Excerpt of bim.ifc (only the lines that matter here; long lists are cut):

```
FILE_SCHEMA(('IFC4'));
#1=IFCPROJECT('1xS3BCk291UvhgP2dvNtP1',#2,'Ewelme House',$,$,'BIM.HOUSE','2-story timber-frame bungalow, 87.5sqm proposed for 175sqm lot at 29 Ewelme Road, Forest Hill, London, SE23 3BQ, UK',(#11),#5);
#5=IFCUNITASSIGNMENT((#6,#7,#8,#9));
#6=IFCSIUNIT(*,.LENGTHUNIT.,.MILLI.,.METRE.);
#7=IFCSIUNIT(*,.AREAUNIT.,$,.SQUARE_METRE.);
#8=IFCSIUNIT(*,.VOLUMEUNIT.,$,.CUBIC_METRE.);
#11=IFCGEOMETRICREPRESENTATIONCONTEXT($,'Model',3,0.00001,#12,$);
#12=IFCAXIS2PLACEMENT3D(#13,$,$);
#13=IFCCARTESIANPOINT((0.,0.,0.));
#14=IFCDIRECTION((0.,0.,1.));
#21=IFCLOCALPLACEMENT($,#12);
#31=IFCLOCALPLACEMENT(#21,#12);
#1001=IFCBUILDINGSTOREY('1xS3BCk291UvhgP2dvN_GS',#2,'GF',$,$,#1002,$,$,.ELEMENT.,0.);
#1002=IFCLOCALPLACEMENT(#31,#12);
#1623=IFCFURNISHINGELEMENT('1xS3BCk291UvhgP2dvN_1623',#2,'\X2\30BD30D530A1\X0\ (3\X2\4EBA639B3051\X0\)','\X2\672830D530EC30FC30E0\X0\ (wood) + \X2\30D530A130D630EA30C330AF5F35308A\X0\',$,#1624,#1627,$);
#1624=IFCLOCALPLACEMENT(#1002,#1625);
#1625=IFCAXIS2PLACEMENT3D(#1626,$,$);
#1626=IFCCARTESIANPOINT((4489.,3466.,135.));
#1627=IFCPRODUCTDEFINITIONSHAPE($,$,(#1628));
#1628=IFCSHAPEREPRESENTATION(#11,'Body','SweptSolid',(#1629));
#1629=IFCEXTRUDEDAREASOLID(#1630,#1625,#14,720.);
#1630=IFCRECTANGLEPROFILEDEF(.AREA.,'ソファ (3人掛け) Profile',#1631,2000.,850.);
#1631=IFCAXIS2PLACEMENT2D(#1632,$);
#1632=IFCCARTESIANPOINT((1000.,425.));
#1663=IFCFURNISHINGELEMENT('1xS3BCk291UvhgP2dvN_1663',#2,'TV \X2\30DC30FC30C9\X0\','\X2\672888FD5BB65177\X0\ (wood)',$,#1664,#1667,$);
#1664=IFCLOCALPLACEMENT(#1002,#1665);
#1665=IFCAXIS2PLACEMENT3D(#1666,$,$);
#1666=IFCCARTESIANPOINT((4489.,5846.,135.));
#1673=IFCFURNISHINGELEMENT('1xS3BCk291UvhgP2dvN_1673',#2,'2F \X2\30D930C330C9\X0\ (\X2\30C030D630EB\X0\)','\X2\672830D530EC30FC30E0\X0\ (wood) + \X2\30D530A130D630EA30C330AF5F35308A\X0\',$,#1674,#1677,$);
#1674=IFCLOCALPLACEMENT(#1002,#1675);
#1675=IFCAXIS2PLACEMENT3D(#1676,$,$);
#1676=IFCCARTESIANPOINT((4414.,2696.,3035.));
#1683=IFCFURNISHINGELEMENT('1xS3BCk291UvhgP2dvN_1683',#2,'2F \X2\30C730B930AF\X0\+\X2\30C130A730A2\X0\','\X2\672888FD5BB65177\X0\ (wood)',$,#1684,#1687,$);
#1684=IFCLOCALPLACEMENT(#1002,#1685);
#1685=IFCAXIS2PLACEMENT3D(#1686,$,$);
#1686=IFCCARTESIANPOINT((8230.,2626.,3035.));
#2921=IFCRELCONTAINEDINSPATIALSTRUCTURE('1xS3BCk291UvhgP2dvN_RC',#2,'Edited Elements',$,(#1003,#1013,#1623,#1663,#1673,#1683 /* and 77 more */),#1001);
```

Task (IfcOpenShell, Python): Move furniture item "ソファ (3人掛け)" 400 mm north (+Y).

```python
import ifcopenshell
import ifcopenshell.api.geometry
import ifcopenshell.util.placement
import ifcopenshell.util.unit

model = ifcopenshell.open("bim.ifc")
unit_scale = ifcopenshell.util.unit.calculate_unit_scale(model)

item = model.by_guid("1xS3BCk291UvhgP2dvN_1623")
matrix = ifcopenshell.util.placement.get_local_placement(item.ObjectPlacement)
matrix[1, 3] += 0.4 / unit_scale
ifcopenshell.api.geometry.edit_object_placement(model, product=item, matrix=matrix, is_si=False)

print(ifcopenshell.util.placement.get_local_placement(item.ObjectPlacement).round(3) + 0.0)

model.write("bim_edited.ifc")
```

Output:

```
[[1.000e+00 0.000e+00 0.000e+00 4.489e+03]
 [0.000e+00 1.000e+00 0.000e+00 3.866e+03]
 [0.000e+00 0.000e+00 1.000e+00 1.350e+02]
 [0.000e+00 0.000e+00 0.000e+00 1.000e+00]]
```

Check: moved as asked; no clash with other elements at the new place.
